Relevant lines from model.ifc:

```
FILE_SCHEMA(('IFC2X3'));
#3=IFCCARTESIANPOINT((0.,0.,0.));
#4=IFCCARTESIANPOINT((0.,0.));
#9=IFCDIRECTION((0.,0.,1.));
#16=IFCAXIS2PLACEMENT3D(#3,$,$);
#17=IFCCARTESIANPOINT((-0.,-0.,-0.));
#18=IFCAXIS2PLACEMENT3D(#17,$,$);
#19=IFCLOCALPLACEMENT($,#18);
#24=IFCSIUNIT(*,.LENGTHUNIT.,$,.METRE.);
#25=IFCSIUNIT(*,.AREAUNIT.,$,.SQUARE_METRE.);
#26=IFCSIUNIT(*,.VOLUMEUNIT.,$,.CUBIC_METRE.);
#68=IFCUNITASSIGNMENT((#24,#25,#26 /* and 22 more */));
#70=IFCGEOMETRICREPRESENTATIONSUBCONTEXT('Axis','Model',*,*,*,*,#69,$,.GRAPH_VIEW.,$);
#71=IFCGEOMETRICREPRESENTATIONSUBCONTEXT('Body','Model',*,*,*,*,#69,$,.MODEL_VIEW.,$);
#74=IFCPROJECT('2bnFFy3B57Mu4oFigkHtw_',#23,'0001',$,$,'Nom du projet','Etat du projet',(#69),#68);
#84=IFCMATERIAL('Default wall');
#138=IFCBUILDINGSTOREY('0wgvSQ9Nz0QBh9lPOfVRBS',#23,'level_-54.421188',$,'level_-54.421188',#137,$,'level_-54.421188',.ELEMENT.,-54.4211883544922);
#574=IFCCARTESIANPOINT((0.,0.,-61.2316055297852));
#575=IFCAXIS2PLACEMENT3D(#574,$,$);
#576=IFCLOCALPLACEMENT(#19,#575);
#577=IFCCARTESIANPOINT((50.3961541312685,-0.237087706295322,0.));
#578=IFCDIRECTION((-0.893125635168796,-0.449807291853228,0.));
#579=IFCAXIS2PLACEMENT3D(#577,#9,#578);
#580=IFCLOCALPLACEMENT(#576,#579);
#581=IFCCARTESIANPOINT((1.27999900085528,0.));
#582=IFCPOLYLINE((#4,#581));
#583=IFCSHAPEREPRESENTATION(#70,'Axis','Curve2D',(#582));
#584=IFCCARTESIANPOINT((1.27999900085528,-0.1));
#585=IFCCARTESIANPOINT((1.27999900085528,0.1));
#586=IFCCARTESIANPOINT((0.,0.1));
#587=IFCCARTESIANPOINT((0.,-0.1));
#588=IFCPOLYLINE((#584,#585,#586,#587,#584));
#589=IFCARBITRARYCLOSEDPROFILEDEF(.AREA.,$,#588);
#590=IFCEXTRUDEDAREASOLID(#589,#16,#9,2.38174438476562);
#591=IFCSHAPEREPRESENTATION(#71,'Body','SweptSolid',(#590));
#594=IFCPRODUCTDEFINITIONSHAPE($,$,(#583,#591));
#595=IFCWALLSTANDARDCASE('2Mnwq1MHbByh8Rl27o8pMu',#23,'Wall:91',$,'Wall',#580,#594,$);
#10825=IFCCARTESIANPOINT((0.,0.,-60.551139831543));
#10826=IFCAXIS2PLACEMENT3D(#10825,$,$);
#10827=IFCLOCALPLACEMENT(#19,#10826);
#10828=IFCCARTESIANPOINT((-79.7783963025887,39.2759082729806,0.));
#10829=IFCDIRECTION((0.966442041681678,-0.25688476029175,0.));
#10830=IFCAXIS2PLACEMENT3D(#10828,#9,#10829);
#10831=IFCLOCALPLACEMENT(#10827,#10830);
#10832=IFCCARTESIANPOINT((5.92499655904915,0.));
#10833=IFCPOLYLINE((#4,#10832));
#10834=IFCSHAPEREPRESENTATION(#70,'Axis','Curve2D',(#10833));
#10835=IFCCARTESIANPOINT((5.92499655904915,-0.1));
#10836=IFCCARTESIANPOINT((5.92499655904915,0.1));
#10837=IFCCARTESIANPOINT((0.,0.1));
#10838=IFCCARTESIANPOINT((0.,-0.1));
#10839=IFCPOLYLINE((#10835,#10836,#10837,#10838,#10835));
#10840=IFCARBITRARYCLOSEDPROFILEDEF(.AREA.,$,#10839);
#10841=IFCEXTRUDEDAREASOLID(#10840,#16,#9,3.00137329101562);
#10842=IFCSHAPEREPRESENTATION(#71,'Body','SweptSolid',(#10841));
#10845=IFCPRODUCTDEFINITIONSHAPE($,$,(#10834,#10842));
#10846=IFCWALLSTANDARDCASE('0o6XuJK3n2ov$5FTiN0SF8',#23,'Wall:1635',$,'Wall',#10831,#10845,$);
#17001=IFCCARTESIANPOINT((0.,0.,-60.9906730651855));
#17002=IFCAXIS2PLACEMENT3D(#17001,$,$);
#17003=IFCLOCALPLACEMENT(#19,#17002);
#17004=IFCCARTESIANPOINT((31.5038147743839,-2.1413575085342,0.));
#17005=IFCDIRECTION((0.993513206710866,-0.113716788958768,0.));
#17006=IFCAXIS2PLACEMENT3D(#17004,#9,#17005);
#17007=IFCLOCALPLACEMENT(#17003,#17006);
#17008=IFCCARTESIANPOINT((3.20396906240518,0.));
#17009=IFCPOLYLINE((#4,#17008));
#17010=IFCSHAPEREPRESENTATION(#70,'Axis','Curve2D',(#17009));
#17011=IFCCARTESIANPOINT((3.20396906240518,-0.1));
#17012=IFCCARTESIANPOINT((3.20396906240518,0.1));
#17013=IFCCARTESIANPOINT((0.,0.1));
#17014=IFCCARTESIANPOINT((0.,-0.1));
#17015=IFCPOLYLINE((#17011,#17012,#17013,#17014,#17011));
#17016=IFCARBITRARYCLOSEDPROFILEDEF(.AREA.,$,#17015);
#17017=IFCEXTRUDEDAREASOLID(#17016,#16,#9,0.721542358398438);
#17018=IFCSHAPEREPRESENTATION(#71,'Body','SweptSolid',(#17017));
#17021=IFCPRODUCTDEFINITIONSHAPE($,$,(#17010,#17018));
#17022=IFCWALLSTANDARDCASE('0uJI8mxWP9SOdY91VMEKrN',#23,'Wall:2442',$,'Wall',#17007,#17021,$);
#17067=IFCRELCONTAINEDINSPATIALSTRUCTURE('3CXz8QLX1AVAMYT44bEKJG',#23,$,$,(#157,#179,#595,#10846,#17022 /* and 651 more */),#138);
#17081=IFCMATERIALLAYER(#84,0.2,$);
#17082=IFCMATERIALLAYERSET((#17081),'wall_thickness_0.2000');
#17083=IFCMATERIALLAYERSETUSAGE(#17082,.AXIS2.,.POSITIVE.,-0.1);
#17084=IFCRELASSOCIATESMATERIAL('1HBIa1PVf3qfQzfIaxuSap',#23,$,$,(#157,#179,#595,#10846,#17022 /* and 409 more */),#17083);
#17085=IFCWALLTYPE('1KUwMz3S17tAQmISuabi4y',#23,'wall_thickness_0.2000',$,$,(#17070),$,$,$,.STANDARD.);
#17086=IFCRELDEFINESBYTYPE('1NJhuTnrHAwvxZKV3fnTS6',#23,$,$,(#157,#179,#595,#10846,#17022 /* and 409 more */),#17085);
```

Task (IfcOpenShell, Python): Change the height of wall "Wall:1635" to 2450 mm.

```python
import ifcopenshell
import ifcopenshell.geom
import ifcopenshell.util.representation
import ifcopenshell.util.shape

model = ifcopenshell.open("model.ifc")
settings = ifcopenshell.geom.settings()


def volume(element):
    """Net volume in cubic metres, openings subtracted."""
    shape = ifcopenshell.geom.create_shape(settings, element)
    return ifcopenshell.util.shape.get_volume(shape.geometry)


wall = model.by_id(10846)
before = volume(wall)

body = ifcopenshell.util.representation.get_representation(wall, "Model", "Body")
solid = body.Items[0]
old_height = solid.Depth
solid.Depth = 2.45
after = volume(wall)

print(f"height {old_height:g} -> {solid.Depth:g}, volume {before:.3f} -> {after:.3f} m3")

model.write("model_rev.ifc")
```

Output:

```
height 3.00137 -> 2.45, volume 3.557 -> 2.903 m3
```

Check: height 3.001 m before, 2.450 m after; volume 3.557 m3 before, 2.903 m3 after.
